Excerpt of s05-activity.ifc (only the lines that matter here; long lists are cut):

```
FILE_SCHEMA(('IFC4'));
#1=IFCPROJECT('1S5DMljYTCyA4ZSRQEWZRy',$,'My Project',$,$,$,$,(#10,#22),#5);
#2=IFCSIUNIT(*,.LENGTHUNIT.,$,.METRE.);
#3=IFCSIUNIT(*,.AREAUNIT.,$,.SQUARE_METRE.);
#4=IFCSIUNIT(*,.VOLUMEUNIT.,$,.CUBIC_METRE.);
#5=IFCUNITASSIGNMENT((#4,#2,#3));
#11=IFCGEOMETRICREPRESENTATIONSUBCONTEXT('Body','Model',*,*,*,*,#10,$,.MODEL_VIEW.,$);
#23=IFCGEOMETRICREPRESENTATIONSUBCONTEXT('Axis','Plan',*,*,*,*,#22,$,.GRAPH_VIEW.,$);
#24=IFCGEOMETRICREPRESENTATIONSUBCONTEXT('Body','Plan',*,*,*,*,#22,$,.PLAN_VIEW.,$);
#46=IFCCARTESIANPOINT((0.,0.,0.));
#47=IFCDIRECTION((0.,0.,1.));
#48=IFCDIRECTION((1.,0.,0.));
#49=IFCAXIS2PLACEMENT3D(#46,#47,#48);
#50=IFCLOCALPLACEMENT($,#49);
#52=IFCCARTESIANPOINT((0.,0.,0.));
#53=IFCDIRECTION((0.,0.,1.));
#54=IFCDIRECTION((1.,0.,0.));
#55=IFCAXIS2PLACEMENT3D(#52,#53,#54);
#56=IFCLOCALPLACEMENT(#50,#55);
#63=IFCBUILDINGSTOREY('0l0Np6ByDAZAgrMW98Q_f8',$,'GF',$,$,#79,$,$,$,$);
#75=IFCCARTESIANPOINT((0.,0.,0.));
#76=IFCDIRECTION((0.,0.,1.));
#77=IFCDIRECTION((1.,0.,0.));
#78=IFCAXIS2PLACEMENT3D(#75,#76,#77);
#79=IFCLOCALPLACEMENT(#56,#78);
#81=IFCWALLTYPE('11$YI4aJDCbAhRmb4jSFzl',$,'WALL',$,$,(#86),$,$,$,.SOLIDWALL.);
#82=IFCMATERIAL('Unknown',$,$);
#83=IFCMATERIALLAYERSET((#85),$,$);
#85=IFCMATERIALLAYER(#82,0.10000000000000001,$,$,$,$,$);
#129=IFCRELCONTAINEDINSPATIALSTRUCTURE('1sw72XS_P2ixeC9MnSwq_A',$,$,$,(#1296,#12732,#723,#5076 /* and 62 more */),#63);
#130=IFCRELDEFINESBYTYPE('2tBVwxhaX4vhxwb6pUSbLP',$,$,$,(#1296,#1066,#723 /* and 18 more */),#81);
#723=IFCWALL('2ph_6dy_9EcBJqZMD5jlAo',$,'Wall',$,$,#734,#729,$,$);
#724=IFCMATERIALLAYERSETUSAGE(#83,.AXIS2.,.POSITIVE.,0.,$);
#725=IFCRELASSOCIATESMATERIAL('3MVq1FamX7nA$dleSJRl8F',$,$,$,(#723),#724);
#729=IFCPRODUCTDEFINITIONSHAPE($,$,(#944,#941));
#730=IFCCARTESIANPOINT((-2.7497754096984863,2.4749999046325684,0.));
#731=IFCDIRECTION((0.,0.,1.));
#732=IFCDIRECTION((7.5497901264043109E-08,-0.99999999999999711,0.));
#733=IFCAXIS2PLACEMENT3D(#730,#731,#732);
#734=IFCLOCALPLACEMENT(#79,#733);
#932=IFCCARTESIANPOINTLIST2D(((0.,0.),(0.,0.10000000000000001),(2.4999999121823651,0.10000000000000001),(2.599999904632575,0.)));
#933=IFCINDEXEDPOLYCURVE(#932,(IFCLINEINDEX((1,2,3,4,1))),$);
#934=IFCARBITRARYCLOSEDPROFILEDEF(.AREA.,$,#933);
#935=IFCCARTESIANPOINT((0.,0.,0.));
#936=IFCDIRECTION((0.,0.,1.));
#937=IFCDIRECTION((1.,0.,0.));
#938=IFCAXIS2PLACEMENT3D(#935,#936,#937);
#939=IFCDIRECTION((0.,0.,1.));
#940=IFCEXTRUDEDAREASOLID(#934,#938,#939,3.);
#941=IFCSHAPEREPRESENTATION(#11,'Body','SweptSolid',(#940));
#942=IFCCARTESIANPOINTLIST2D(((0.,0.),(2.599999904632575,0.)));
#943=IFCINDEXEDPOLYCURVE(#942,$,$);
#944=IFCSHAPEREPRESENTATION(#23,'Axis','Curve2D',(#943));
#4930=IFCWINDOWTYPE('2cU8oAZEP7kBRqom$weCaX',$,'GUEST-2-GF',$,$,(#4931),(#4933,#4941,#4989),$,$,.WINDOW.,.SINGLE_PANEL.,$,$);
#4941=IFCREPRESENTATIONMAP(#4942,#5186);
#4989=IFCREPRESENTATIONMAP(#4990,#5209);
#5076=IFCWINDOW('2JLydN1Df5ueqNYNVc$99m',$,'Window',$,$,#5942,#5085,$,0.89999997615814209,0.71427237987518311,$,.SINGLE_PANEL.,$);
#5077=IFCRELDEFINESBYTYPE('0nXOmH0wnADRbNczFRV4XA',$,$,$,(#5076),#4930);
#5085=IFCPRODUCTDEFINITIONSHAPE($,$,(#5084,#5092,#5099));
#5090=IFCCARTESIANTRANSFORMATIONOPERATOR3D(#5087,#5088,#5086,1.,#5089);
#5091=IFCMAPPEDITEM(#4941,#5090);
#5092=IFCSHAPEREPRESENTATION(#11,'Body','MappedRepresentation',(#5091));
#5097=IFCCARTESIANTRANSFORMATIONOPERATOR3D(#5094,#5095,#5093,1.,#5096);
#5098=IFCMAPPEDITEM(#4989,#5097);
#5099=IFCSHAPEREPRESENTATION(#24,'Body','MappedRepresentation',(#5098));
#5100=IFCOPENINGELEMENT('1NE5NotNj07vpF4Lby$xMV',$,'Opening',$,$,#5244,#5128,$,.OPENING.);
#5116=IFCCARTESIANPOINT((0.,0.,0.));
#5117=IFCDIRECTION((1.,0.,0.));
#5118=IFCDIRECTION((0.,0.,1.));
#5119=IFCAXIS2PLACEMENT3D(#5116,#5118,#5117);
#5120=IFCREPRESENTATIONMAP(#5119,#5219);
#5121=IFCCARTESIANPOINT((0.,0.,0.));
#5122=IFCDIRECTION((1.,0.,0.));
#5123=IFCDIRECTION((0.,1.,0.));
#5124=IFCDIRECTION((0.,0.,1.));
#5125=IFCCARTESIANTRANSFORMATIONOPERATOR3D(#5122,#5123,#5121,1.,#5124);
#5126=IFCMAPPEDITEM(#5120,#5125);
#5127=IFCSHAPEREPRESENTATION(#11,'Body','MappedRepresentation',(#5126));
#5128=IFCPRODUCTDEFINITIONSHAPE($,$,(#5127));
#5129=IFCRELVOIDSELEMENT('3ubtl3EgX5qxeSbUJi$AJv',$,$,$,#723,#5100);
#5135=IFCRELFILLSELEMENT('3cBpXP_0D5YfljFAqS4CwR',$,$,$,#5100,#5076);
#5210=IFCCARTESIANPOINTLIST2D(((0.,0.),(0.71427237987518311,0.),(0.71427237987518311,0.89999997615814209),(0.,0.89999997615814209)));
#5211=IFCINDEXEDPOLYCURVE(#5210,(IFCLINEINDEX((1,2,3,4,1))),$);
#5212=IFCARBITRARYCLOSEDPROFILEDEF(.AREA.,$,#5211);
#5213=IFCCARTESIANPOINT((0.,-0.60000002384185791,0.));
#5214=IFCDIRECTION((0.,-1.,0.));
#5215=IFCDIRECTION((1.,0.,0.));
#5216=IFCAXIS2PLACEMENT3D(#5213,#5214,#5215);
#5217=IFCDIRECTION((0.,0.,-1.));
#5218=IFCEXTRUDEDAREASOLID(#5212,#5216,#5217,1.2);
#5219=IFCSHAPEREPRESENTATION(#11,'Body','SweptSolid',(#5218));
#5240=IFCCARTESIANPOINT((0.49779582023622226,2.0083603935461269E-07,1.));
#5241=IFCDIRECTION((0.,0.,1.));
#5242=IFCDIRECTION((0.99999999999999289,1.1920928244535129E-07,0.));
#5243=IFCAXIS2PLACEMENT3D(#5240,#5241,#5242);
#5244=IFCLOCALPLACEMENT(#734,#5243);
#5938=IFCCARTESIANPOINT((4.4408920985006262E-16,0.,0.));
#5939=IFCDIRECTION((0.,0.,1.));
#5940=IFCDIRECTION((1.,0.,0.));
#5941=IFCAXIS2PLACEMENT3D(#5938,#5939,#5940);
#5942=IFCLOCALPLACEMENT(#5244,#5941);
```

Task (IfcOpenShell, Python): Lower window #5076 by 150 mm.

```python
import numpy as np
import ifcopenshell
import ifcopenshell.api.geometry
import ifcopenshell.util.placement
import ifcopenshell.util.unit

model = ifcopenshell.open("s05-activity.ifc")
unit_scale = ifcopenshell.util.unit.calculate_unit_scale(model)

window = model.by_guid("2JLydN1Df5ueqNYNVc$99m")
opening = window.FillsVoids[0].RelatingOpeningElement
dz = -0.15 / unit_scale

shift = np.array([0.0, 0.0, dz])
# The window is placed relative to its opening, so it follows when the opening moves.
matrix = ifcopenshell.util.placement.get_local_placement(opening.ObjectPlacement)
matrix[:3, 3] += shift
ifcopenshell.api.geometry.edit_object_placement(
    model, product=opening, matrix=matrix, is_si=False, should_transform_children=True
)

print(f"moved by {dz * unit_scale:+.3f} m")

model.write("s05-activity_edited.ifc")
```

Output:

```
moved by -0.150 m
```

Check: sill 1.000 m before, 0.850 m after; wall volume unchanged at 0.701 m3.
